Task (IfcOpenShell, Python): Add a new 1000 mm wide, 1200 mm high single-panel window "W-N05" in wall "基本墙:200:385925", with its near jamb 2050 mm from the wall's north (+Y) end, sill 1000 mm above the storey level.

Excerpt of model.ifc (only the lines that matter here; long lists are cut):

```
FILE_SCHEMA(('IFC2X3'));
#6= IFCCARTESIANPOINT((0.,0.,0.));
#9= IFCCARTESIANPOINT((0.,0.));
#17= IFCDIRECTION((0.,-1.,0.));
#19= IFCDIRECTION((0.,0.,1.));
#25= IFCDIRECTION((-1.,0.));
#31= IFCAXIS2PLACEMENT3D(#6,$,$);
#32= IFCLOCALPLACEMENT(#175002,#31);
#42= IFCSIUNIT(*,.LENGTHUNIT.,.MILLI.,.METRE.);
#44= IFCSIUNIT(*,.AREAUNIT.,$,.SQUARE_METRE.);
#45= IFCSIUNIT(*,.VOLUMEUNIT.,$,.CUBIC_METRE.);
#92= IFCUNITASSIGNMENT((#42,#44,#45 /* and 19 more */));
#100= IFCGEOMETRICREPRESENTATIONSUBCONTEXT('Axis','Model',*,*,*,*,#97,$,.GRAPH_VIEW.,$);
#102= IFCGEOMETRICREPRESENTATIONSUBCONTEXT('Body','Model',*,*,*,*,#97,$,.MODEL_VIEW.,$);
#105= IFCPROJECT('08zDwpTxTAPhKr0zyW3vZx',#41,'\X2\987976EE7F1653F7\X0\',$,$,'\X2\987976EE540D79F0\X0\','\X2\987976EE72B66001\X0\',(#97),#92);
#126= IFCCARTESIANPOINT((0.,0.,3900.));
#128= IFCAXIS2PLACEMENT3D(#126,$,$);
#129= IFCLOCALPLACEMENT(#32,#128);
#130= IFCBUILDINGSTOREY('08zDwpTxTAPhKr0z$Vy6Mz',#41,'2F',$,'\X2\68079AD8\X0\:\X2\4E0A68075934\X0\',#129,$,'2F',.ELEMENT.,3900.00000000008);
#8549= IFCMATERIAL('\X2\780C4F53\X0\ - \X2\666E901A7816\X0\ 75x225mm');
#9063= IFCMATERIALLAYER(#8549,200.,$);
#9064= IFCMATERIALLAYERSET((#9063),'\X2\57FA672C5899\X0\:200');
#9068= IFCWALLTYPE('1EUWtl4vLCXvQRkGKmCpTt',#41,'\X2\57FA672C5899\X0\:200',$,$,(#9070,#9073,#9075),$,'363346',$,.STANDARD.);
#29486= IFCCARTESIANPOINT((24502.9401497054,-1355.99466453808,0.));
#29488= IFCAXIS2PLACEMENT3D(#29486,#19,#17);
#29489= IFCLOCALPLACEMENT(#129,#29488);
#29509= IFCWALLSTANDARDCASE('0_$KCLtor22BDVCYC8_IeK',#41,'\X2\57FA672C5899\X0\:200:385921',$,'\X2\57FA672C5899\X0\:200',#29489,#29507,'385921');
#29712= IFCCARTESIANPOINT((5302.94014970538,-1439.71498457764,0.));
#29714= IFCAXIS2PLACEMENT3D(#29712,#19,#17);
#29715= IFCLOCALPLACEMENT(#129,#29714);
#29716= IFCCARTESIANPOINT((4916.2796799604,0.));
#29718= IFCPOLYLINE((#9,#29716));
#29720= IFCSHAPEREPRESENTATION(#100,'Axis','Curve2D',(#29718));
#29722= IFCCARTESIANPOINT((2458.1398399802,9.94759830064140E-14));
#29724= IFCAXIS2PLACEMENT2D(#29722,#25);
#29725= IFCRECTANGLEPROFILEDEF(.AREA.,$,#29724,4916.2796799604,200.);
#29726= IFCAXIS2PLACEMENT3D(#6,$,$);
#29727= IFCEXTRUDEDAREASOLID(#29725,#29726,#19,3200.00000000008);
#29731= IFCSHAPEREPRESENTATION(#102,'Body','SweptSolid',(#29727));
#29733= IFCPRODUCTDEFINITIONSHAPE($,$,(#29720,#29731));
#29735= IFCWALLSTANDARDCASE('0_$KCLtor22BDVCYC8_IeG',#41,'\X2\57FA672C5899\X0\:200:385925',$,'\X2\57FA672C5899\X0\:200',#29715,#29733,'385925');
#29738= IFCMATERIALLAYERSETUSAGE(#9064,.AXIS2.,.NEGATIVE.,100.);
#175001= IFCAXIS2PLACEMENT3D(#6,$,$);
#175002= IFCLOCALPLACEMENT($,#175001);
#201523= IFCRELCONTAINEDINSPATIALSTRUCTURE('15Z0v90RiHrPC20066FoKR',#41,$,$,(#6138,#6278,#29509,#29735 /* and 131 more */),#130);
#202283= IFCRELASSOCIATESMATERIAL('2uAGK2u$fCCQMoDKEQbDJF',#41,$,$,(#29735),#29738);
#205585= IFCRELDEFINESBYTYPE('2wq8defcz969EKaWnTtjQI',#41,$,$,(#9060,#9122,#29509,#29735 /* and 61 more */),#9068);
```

```python
import numpy as np
import ifcopenshell
import ifcopenshell.api.feature
import ifcopenshell.api.geometry
import ifcopenshell.api.root
import ifcopenshell.api.spatial
import ifcopenshell.api.type
import ifcopenshell.geom
import ifcopenshell.util.element
import ifcopenshell.util.placement
import ifcopenshell.util.representation
import ifcopenshell.util.shape
import ifcopenshell.util.unit

model = ifcopenshell.open("model.ifc")
unit_scale = ifcopenshell.util.unit.calculate_unit_scale(model)
settings = ifcopenshell.geom.settings()


def volume(element):
    """Net volume in cubic metres, openings subtracted."""
    shape = ifcopenshell.geom.create_shape(settings, element)
    return ifcopenshell.util.shape.get_volume(shape.geometry)


wall = model.by_id(29735)
storey = ifcopenshell.util.element.get_container(wall, ifc_class="IfcBuildingStorey")
context = ifcopenshell.util.representation.get_context(model, "Model", "Body", "MODEL_VIEW")
before = volume(wall)

width, height, from_end, sill = 1, 1.2, 2.05, 1  # metres

# The wall runs along its own X axis, and the end named is its -X end.
wall_shape = ifcopenshell.geom.create_shape(settings, wall)
x, y, z = ifcopenshell.util.shape.get_vertices(wall_shape.geometry).T
start = x.min() + from_end
face, thickness = float(y.min()), float(y.max() - y.min())
wall_matrix = ifcopenshell.util.placement.get_local_placement(wall.ObjectPlacement)
level = ifcopenshell.util.placement.get_local_placement(storey.ObjectPlacement)[2, 3]


def in_wall(x, y):
    """Placement at x, y metres in the wall's axes, at sill height."""
    matrix = wall_matrix.copy()
    matrix[:, 3] = wall_matrix @ np.array([x / unit_scale, y / unit_scale, 0.0, 1.0])
    matrix[2, 3] = level + sill / unit_scale
    return matrix


# Opening: a box that overshoots both wall faces by 50 mm.
opening = ifcopenshell.api.root.create_entity(model, ifc_class="IfcOpeningElement")
box = ifcopenshell.api.geometry.add_wall_representation(
    model, context=context, length=width, height=height, thickness=thickness + 0.1
)
ifcopenshell.api.geometry.assign_representation(model, product=opening, representation=box)
ifcopenshell.api.geometry.edit_object_placement(model, product=opening, matrix=in_wall(start, face - 0.05), is_si=False)
ifcopenshell.api.feature.add_feature(model, feature=opening, element=wall)

window = ifcopenshell.api.root.create_entity(model, ifc_class="IfcWindow", name="W-N05")
window.OverallWidth, window.OverallHeight = width / unit_scale, height / unit_scale
body = ifcopenshell.api.geometry.add_window_representation(
    model,
    context=context,
    overall_width=window.OverallWidth,
    overall_height=window.OverallHeight,
    partition_type="SINGLE_PANEL",
)
ifcopenshell.api.geometry.assign_representation(model, product=window, representation=body)
ifcopenshell.api.spatial.assign_container(model, products=[window], relating_structure=storey)
fills = ifcopenshell.api.feature.add_filling(model, opening=opening, element=window)
fills.OwnerHistory = window.OwnerHistory  # required in IFC2X3

# IFC2X3 keeps the operation on the window style.
style = ifcopenshell.api.root.create_entity(model, ifc_class="IfcWindowStyle", name="W-N05")
style.OperationType, style.ConstructionType = "SINGLE_PANEL", "NOTDEFINED"
style.ParameterTakesPrecedence = style.Sizeable = False
ifcopenshell.api.type.assign_type(model, related_objects=[window], relating_type=style)

# Centre the window in the wall's thickness.
ifcopenshell.api.geometry.edit_object_placement(model, product=window, matrix=in_wall(start, face), is_si=False)
window_shape = ifcopenshell.geom.create_shape(settings, window)
depth = ifcopenshell.util.shape.get_vertices(window_shape.geometry)[:, 1]
offset = face + thickness / 2 - (depth.min() + depth.max()) / 2
ifcopenshell.api.geometry.edit_object_placement(model, product=window, matrix=in_wall(start, offset), is_si=False)

after = volume(wall)

print(f"wall volume {before:.3f} -> {after:.3f} m3")

model.write("model_edited.ifc")
```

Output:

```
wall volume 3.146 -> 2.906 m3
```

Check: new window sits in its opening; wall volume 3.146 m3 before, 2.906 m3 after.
